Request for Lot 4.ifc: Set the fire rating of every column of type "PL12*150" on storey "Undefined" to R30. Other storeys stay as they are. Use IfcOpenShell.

First a look at what the model holds.

```python
import ifcopenshell
import ifcopenshell.util.element

model = ifcopenshell.open("Lot 4.ifc")
print(model.schema)
storey = next(s for s in model.by_type("IfcBuildingStorey") if s.Name == "Undefined")
columns = [e for e in ifcopenshell.util.element.get_decomposition(storey) if e.is_a("IfcColumn")]
seen = {}
for e in columns:
    element_type = ifcopenshell.util.element.get_type(e)
    key = (element_type.Name if element_type != e and element_type else None, ifcopenshell.util.element.get_pset(e, "Pset_ColumnCommon", "FireRating"))
    seen[key] = seen.get(key, 0) + 1
for (name, value), count in sorted(seen.items(), key=str):
    print(count, "x", name, "|", value)
```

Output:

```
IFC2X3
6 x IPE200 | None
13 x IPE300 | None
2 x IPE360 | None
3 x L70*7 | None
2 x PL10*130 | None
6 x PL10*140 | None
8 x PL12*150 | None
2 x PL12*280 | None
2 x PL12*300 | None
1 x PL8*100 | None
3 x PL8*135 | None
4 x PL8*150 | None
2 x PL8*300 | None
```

```python
import ifcopenshell
import ifcopenshell.api.pset
import ifcopenshell.util.element

model = ifcopenshell.open("Lot 4.ifc")

storey = next(s for s in model.by_type("IfcBuildingStorey") if s.Name == "Undefined")
columns = [e for e in ifcopenshell.util.element.get_decomposition(storey) if e.is_a("IfcColumn")]

count = 0
for e in columns:
    element_type = ifcopenshell.util.element.get_type(e)
    if element_type in (None, e) or element_type.Name != "PL12*150":
        continue
    found = ifcopenshell.util.element.get_pset(e, "Pset_ColumnCommon", should_inherit=False)
    if found:
        pset = model.by_id(found["id"])
        if len(ifcopenshell.util.element.get_elements_by_pset(pset)) > 1:
            pset = ifcopenshell.api.pset.unshare_pset(model, products=[e], pset=pset)[0]
    else:
        pset = ifcopenshell.api.pset.add_pset(model, product=e, name="Pset_ColumnCommon")
    ifcopenshell.api.pset.edit_pset(model, pset=pset, properties={"FireRating": "R30"})
    count += 1

print(count, "columns updated")

model.write("Lot 4_rev.ifc")
```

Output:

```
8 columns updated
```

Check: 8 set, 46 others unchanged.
